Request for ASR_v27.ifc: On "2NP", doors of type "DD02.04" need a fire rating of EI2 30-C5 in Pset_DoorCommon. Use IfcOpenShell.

First a look at what the model holds.

```python
import ifcopenshell
import ifcopenshell.util.element

model = ifcopenshell.open("ASR_v27.ifc")
print(model.schema)
storey = next(s for s in model.by_type("IfcBuildingStorey") if s.Name == "2NP")
doors = [e for e in ifcopenshell.util.element.get_decomposition(storey) if e.is_a("IfcDoor")]
seen = {}
for e in doors:
    element_type = ifcopenshell.util.element.get_type(e)
    key = (element_type.Name if element_type != e and element_type else None, ifcopenshell.util.element.get_pset(e, "Pset_DoorCommon", "FireRating"))
    seen[key] = seen.get(key, 0) + 1
for (name, value), count in sorted(seen.items(), key=str):
    print(count, "x", name, "|", value)
```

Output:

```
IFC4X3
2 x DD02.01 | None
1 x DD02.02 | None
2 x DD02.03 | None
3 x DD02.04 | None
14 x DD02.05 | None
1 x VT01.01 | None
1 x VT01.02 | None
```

```python
import ifcopenshell
import ifcopenshell.api.pset
import ifcopenshell.util.element

model = ifcopenshell.open("ASR_v27.ifc")

storey = next(s for s in model.by_type("IfcBuildingStorey") if s.Name == "2NP")
doors = [e for e in ifcopenshell.util.element.get_decomposition(storey) if e.is_a("IfcDoor")]

count = 0
for e in doors:
    element_type = ifcopenshell.util.element.get_type(e)
    if element_type in (None, e) or element_type.Name != "DD02.04":
        continue
    # add_pset returns the element's existing set when there is one.
    pset = ifcopenshell.api.pset.add_pset(model, product=e, name="Pset_DoorCommon")
    ifcopenshell.api.pset.edit_pset(model, pset=pset, properties={"FireRating": "EI2 30-C5"})
    count += 1

print(count, "doors updated")

model.write("ASR_v27_rev.ifc")
```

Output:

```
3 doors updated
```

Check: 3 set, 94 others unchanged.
